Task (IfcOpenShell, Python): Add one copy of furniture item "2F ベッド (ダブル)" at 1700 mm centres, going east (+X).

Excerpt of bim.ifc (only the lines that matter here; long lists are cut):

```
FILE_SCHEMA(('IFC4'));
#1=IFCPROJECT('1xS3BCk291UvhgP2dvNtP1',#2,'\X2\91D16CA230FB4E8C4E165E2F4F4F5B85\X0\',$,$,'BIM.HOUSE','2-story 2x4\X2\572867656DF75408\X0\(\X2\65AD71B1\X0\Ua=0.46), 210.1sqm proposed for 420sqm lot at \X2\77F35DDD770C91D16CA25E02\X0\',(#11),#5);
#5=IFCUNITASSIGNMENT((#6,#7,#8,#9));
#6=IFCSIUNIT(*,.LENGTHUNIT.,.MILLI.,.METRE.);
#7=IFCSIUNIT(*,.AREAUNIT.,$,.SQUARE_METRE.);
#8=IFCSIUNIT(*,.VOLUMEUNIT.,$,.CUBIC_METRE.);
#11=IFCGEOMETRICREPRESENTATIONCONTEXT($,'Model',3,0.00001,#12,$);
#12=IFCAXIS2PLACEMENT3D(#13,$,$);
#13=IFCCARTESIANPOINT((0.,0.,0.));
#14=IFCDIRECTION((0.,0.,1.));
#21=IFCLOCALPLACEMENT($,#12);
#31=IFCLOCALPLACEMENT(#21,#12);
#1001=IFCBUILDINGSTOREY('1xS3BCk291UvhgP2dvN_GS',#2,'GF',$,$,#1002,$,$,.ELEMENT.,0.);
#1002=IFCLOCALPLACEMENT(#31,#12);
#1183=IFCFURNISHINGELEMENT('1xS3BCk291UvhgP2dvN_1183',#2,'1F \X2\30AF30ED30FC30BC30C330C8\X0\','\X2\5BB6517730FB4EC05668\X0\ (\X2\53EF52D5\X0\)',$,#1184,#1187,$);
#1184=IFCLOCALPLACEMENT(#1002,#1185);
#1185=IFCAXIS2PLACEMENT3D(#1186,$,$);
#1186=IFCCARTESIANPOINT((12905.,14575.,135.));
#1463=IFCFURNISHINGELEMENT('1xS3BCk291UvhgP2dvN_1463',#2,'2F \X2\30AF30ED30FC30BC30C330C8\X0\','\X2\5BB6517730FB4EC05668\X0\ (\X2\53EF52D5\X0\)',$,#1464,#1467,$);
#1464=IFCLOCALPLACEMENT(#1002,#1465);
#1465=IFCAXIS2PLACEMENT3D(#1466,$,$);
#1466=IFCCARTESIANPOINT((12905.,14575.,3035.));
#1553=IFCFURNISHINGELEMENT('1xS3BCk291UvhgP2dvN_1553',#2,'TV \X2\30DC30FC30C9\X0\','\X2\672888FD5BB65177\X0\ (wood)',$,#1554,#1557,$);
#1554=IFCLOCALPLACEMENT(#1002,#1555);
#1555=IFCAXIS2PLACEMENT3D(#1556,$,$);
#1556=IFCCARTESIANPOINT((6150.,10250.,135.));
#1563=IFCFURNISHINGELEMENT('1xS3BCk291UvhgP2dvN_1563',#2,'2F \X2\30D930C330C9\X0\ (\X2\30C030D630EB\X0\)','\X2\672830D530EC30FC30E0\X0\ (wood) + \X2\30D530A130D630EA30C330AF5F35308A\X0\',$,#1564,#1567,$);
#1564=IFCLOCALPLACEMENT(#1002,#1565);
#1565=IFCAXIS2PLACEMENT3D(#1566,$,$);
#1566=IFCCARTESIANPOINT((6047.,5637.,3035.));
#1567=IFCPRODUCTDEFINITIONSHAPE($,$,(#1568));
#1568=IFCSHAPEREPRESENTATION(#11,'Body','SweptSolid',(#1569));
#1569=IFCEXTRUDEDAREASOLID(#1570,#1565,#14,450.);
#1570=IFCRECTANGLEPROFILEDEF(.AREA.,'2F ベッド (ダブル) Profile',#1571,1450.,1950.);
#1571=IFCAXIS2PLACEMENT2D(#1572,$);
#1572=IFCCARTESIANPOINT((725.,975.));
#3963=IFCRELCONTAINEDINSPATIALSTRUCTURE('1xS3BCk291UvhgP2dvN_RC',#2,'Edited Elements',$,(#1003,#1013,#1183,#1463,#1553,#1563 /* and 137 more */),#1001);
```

```python
import numpy as np
import ifcopenshell
import ifcopenshell.api.geometry
import ifcopenshell.api.root
import ifcopenshell.util.element
import ifcopenshell.util.placement

model = ifcopenshell.open("bim.ifc")


def reuse_history(source, copy):
    """copy_class also copies each property set's owner history, people and application; keep the originals."""
    for rel in copy.IsDefinedBy:
        if rel.is_a("IfcRelDefinesByProperties") and (history := rel.RelatingPropertyDefinition.OwnerHistory):
            rel.RelatingPropertyDefinition.OwnerHistory = source.OwnerHistory
            ifcopenshell.util.element.remove_deep2(model, history)


source = model.by_guid("1xS3BCk291UvhgP2dvN_1563")
base = ifcopenshell.util.placement.get_local_placement(source.ObjectPlacement)
step = np.array([1.0, 0.0, 0.0]) * 1700.0

for i in range(1, 2):
    copy = ifcopenshell.api.root.copy_class(model, product=source)
    copy.Representation = ifcopenshell.util.element.copy_deep(
        model, source.Representation, exclude=["IfcGeometricRepresentationContext", "IfcRepresentationMap"]
    )
    reuse_history(source, copy)
    matrix = base.copy()
    matrix[:3, 3] += i * step
    print("added at", matrix[:3, 3].round(3) + 0.0)
    ifcopenshell.api.geometry.edit_object_placement(model, product=copy, matrix=matrix, is_si=False)

model.write("bim_edited.ifc")
```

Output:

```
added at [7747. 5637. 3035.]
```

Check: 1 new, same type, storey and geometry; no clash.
